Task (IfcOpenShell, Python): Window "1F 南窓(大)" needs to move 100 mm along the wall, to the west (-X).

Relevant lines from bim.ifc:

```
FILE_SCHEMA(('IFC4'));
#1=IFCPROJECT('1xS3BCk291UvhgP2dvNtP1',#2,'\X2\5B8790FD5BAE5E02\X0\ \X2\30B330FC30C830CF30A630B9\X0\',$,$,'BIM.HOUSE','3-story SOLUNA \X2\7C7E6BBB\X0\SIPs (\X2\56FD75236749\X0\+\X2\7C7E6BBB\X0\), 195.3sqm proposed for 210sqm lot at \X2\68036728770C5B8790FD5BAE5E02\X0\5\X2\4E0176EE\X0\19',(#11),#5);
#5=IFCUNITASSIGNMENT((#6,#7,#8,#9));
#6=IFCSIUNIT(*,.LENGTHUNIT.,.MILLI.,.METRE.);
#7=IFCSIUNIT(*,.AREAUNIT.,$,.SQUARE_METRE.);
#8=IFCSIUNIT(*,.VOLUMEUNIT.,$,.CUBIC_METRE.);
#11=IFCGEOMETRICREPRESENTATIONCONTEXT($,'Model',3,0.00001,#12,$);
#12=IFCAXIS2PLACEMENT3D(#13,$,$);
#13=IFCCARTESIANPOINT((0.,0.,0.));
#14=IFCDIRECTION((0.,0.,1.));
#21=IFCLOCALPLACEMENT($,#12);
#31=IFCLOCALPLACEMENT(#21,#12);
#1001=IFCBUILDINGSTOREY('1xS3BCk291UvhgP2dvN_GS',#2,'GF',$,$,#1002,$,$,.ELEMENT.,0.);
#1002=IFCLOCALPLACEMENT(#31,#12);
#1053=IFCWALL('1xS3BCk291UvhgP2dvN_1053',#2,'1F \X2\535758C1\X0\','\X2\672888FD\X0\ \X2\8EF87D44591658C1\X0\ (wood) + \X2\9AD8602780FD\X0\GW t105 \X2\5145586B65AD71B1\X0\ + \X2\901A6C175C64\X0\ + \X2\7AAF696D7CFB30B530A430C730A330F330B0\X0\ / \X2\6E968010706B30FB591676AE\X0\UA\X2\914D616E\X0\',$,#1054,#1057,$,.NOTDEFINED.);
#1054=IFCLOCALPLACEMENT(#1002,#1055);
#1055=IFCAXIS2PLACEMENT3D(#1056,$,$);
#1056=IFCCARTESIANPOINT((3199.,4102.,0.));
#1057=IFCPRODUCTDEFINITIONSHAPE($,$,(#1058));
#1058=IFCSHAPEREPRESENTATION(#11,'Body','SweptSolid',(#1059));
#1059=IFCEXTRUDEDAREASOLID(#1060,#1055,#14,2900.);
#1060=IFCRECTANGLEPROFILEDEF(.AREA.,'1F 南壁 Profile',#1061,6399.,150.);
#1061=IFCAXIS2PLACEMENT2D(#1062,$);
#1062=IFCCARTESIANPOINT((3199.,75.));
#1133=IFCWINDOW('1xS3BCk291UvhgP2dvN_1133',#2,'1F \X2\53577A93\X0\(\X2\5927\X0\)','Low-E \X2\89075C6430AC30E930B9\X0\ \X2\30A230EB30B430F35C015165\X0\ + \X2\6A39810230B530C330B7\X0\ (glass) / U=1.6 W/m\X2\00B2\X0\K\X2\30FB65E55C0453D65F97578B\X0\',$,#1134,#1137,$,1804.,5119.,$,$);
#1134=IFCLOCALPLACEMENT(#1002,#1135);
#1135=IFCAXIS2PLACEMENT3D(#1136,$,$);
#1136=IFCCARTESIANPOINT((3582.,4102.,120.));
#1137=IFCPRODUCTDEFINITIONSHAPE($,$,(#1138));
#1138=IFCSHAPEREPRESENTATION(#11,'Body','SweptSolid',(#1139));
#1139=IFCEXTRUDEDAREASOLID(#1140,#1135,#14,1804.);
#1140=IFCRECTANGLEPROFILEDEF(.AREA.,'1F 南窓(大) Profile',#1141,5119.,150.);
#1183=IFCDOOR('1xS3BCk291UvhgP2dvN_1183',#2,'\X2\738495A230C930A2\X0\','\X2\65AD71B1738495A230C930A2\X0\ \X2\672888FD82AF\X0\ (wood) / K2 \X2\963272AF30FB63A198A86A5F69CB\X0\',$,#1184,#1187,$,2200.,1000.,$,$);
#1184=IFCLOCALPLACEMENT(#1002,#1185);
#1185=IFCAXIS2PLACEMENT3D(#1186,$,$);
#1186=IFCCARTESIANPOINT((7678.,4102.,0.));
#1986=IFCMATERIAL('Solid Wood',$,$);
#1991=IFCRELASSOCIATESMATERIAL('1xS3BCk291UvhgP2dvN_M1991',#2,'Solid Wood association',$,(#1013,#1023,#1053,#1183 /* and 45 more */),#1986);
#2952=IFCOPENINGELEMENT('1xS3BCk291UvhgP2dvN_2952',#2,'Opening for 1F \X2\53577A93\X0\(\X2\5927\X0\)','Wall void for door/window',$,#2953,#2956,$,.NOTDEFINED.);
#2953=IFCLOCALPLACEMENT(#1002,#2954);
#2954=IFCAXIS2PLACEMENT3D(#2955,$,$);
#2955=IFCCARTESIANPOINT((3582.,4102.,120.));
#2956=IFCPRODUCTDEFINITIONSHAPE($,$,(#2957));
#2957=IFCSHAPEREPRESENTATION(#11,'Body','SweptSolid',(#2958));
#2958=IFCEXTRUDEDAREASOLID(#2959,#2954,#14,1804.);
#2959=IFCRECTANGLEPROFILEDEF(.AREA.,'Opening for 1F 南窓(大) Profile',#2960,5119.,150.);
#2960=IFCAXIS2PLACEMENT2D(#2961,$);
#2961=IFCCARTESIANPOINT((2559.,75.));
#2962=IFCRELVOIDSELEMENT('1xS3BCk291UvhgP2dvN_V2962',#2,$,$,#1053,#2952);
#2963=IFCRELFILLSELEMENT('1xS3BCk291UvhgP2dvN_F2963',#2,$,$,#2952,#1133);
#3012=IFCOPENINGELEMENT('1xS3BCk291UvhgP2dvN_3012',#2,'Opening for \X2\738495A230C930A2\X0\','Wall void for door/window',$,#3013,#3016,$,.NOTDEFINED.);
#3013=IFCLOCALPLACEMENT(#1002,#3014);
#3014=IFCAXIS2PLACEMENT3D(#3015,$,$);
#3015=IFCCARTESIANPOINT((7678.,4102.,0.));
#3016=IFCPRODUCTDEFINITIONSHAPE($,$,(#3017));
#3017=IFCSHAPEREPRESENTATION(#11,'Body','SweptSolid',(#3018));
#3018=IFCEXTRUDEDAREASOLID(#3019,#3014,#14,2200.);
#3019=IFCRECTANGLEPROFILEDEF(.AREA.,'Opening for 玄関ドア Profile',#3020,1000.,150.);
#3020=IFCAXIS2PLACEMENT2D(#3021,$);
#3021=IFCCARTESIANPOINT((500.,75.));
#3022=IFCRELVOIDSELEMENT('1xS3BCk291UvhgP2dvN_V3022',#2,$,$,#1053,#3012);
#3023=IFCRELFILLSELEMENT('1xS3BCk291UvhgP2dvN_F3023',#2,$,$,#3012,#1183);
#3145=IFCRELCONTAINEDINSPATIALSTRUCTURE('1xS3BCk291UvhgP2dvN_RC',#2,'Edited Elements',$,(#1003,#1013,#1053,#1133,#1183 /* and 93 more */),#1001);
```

```python
import ifcopenshell
import ifcopenshell.api.geometry
import ifcopenshell.util.placement
import ifcopenshell.util.unit

model = ifcopenshell.open("bim.ifc")
unit_scale = ifcopenshell.util.unit.calculate_unit_scale(model)

window = model.by_guid("1xS3BCk291UvhgP2dvN_1133")
opening = window.FillsVoids[0].RelatingOpeningElement
wall = opening.VoidsElements[0].RelatingBuildingElement

wall_matrix = ifcopenshell.util.placement.get_local_placement(wall.ObjectPlacement)
shift = wall_matrix[:3, 0] * -0.1 / unit_scale
before = ifcopenshell.util.placement.get_local_placement(window.ObjectPlacement)[:3, 3].copy()

# The window is not placed relative to its opening, so move both.
for product in (opening, window):
    matrix = ifcopenshell.util.placement.get_local_placement(product.ObjectPlacement)
    matrix[:3, 3] += shift
    ifcopenshell.api.geometry.edit_object_placement(model, product=product, matrix=matrix, is_si=False)

after = ifcopenshell.util.placement.get_local_placement(window.ObjectPlacement)[:3, 3]
print("window moved by", (after - before).round(3) + 0.0)

model.write("bim_rev.ifc")
```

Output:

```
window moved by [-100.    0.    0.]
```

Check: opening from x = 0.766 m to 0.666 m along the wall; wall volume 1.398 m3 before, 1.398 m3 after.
